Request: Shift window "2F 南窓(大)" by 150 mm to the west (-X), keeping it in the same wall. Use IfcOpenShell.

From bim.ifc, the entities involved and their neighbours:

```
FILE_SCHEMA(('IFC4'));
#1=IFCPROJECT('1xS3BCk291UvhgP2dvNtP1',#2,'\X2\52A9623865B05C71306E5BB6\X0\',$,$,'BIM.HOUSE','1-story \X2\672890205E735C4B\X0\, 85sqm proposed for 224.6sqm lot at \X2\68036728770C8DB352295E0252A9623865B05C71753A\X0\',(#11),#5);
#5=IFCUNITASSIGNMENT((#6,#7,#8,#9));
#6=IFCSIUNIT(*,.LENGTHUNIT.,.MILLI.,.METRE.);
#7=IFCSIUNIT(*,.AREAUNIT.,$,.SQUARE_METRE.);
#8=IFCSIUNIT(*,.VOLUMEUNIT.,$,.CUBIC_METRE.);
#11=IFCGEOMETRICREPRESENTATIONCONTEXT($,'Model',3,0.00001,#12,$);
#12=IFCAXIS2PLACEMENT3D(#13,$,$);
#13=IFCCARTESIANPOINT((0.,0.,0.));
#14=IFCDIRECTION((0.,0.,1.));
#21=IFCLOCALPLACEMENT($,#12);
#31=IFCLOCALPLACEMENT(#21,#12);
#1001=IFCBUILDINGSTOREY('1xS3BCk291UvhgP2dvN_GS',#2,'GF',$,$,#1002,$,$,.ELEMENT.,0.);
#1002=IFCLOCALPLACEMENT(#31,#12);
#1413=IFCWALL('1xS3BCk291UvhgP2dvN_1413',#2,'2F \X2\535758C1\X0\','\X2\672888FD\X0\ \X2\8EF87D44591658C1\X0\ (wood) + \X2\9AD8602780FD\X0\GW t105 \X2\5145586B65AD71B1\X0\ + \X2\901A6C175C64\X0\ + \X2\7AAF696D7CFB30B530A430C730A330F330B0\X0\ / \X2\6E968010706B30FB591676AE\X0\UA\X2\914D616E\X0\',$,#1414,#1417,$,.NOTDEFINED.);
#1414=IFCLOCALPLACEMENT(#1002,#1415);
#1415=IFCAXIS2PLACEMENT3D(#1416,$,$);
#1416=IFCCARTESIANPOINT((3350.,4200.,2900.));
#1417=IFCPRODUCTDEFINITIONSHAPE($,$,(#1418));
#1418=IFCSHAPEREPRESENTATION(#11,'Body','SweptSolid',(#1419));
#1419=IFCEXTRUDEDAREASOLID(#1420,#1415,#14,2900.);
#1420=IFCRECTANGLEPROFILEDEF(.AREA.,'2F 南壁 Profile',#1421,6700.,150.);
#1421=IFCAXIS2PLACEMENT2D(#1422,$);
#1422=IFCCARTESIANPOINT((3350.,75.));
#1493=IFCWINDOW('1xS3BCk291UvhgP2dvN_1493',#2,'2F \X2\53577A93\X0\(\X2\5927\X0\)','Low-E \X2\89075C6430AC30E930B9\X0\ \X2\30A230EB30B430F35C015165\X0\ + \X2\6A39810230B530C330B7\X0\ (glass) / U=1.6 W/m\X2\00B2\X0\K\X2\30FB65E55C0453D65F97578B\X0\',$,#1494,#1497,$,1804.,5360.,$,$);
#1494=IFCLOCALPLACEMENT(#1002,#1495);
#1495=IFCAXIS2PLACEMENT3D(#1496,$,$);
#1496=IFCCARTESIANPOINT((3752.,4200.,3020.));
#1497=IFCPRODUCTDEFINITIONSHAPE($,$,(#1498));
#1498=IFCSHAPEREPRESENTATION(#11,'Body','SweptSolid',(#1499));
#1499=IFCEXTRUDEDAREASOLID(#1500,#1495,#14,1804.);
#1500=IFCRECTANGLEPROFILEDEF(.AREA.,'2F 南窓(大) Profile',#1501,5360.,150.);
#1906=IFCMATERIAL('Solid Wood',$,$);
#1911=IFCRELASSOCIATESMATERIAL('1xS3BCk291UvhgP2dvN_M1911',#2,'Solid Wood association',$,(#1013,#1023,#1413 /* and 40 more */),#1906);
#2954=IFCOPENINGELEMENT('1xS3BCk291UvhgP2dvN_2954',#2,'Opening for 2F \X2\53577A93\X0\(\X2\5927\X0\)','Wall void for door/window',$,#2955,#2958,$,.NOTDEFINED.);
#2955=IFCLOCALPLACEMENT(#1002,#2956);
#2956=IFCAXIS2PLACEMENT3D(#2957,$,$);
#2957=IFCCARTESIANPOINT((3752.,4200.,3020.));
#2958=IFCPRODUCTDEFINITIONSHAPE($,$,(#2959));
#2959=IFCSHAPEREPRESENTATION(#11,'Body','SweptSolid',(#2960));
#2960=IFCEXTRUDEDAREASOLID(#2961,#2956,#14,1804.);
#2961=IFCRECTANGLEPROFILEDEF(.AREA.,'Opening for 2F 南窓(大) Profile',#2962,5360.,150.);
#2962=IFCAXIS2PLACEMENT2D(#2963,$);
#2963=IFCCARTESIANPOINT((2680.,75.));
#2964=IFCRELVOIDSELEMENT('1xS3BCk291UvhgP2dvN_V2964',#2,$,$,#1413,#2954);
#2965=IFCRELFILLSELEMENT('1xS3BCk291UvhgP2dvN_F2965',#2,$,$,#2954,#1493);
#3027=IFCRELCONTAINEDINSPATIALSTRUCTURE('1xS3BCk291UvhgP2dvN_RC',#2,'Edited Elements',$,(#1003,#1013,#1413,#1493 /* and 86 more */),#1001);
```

```python
import ifcopenshell
import ifcopenshell.api.geometry
import ifcopenshell.util.placement
import ifcopenshell.util.unit

model = ifcopenshell.open("bim.ifc")
unit_scale = ifcopenshell.util.unit.calculate_unit_scale(model)

window = model.by_guid("1xS3BCk291UvhgP2dvN_1493")
opening = window.FillsVoids[0].RelatingOpeningElement
wall = opening.VoidsElements[0].RelatingBuildingElement

wall_matrix = ifcopenshell.util.placement.get_local_placement(wall.ObjectPlacement)
shift = wall_matrix[:3, 0] * -0.15 / unit_scale
before = ifcopenshell.util.placement.get_local_placement(window.ObjectPlacement)[:3, 3].copy()

# The window is not placed relative to its opening, so move both.
for product in (opening, window):
    matrix = ifcopenshell.util.placement.get_local_placement(product.ObjectPlacement)
    matrix[:3, 3] += shift
    ifcopenshell.api.geometry.edit_object_placement(model, product=product, matrix=matrix, is_si=False)

after = ifcopenshell.util.placement.get_local_placement(window.ObjectPlacement)[:3, 3]
print("window moved by", (after - before).round(3) + 0.0)

model.write("bim_v2.ifc")
```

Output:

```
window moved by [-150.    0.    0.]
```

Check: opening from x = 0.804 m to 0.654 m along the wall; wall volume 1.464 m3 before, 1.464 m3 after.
